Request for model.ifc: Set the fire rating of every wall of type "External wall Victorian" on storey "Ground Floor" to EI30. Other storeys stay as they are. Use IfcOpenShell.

First a look at what the model holds.

```python
import ifcopenshell
import ifcopenshell.util.element

model = ifcopenshell.open("model.ifc")
print(model.schema)
storey = next(s for s in model.by_type("IfcBuildingStorey") if s.Name == "Ground Floor")
walls = [e for e in ifcopenshell.util.element.get_decomposition(storey) if e.is_a("IfcWall")]
seen = {}
for e in walls:
    element_type = ifcopenshell.util.element.get_type(e)
    key = (element_type.Name if element_type != e and element_type else None, ifcopenshell.util.element.get_pset(e, "Pset_WallCommon", "FireRating"))
    seen[key] = seen.get(key, 0) + 1
for (name, value), count in sorted(seen.items(), key=str):
    print(count, "x", name, "|", value)
```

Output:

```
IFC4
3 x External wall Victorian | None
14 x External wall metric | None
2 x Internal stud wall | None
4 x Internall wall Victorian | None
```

```python
import ifcopenshell
import ifcopenshell.api.pset
import ifcopenshell.util.element

model = ifcopenshell.open("model.ifc")

storey = next(s for s in model.by_type("IfcBuildingStorey") if s.Name == "Ground Floor")
walls = [e for e in ifcopenshell.util.element.get_decomposition(storey) if e.is_a("IfcWall")]

count = 0
for e in walls:
    element_type = ifcopenshell.util.element.get_type(e)
    if element_type in (None, e) or element_type.Name != "External wall Victorian":
        continue
    # add_pset returns the element's existing set when there is one.
    pset = ifcopenshell.api.pset.add_pset(model, product=e, name="Pset_WallCommon")
    ifcopenshell.api.pset.edit_pset(model, pset=pset, properties={"FireRating": "EI30"})
    count += 1

print(count, "walls updated")

model.write("model_edited.ifc")
```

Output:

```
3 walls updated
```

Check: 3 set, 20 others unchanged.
